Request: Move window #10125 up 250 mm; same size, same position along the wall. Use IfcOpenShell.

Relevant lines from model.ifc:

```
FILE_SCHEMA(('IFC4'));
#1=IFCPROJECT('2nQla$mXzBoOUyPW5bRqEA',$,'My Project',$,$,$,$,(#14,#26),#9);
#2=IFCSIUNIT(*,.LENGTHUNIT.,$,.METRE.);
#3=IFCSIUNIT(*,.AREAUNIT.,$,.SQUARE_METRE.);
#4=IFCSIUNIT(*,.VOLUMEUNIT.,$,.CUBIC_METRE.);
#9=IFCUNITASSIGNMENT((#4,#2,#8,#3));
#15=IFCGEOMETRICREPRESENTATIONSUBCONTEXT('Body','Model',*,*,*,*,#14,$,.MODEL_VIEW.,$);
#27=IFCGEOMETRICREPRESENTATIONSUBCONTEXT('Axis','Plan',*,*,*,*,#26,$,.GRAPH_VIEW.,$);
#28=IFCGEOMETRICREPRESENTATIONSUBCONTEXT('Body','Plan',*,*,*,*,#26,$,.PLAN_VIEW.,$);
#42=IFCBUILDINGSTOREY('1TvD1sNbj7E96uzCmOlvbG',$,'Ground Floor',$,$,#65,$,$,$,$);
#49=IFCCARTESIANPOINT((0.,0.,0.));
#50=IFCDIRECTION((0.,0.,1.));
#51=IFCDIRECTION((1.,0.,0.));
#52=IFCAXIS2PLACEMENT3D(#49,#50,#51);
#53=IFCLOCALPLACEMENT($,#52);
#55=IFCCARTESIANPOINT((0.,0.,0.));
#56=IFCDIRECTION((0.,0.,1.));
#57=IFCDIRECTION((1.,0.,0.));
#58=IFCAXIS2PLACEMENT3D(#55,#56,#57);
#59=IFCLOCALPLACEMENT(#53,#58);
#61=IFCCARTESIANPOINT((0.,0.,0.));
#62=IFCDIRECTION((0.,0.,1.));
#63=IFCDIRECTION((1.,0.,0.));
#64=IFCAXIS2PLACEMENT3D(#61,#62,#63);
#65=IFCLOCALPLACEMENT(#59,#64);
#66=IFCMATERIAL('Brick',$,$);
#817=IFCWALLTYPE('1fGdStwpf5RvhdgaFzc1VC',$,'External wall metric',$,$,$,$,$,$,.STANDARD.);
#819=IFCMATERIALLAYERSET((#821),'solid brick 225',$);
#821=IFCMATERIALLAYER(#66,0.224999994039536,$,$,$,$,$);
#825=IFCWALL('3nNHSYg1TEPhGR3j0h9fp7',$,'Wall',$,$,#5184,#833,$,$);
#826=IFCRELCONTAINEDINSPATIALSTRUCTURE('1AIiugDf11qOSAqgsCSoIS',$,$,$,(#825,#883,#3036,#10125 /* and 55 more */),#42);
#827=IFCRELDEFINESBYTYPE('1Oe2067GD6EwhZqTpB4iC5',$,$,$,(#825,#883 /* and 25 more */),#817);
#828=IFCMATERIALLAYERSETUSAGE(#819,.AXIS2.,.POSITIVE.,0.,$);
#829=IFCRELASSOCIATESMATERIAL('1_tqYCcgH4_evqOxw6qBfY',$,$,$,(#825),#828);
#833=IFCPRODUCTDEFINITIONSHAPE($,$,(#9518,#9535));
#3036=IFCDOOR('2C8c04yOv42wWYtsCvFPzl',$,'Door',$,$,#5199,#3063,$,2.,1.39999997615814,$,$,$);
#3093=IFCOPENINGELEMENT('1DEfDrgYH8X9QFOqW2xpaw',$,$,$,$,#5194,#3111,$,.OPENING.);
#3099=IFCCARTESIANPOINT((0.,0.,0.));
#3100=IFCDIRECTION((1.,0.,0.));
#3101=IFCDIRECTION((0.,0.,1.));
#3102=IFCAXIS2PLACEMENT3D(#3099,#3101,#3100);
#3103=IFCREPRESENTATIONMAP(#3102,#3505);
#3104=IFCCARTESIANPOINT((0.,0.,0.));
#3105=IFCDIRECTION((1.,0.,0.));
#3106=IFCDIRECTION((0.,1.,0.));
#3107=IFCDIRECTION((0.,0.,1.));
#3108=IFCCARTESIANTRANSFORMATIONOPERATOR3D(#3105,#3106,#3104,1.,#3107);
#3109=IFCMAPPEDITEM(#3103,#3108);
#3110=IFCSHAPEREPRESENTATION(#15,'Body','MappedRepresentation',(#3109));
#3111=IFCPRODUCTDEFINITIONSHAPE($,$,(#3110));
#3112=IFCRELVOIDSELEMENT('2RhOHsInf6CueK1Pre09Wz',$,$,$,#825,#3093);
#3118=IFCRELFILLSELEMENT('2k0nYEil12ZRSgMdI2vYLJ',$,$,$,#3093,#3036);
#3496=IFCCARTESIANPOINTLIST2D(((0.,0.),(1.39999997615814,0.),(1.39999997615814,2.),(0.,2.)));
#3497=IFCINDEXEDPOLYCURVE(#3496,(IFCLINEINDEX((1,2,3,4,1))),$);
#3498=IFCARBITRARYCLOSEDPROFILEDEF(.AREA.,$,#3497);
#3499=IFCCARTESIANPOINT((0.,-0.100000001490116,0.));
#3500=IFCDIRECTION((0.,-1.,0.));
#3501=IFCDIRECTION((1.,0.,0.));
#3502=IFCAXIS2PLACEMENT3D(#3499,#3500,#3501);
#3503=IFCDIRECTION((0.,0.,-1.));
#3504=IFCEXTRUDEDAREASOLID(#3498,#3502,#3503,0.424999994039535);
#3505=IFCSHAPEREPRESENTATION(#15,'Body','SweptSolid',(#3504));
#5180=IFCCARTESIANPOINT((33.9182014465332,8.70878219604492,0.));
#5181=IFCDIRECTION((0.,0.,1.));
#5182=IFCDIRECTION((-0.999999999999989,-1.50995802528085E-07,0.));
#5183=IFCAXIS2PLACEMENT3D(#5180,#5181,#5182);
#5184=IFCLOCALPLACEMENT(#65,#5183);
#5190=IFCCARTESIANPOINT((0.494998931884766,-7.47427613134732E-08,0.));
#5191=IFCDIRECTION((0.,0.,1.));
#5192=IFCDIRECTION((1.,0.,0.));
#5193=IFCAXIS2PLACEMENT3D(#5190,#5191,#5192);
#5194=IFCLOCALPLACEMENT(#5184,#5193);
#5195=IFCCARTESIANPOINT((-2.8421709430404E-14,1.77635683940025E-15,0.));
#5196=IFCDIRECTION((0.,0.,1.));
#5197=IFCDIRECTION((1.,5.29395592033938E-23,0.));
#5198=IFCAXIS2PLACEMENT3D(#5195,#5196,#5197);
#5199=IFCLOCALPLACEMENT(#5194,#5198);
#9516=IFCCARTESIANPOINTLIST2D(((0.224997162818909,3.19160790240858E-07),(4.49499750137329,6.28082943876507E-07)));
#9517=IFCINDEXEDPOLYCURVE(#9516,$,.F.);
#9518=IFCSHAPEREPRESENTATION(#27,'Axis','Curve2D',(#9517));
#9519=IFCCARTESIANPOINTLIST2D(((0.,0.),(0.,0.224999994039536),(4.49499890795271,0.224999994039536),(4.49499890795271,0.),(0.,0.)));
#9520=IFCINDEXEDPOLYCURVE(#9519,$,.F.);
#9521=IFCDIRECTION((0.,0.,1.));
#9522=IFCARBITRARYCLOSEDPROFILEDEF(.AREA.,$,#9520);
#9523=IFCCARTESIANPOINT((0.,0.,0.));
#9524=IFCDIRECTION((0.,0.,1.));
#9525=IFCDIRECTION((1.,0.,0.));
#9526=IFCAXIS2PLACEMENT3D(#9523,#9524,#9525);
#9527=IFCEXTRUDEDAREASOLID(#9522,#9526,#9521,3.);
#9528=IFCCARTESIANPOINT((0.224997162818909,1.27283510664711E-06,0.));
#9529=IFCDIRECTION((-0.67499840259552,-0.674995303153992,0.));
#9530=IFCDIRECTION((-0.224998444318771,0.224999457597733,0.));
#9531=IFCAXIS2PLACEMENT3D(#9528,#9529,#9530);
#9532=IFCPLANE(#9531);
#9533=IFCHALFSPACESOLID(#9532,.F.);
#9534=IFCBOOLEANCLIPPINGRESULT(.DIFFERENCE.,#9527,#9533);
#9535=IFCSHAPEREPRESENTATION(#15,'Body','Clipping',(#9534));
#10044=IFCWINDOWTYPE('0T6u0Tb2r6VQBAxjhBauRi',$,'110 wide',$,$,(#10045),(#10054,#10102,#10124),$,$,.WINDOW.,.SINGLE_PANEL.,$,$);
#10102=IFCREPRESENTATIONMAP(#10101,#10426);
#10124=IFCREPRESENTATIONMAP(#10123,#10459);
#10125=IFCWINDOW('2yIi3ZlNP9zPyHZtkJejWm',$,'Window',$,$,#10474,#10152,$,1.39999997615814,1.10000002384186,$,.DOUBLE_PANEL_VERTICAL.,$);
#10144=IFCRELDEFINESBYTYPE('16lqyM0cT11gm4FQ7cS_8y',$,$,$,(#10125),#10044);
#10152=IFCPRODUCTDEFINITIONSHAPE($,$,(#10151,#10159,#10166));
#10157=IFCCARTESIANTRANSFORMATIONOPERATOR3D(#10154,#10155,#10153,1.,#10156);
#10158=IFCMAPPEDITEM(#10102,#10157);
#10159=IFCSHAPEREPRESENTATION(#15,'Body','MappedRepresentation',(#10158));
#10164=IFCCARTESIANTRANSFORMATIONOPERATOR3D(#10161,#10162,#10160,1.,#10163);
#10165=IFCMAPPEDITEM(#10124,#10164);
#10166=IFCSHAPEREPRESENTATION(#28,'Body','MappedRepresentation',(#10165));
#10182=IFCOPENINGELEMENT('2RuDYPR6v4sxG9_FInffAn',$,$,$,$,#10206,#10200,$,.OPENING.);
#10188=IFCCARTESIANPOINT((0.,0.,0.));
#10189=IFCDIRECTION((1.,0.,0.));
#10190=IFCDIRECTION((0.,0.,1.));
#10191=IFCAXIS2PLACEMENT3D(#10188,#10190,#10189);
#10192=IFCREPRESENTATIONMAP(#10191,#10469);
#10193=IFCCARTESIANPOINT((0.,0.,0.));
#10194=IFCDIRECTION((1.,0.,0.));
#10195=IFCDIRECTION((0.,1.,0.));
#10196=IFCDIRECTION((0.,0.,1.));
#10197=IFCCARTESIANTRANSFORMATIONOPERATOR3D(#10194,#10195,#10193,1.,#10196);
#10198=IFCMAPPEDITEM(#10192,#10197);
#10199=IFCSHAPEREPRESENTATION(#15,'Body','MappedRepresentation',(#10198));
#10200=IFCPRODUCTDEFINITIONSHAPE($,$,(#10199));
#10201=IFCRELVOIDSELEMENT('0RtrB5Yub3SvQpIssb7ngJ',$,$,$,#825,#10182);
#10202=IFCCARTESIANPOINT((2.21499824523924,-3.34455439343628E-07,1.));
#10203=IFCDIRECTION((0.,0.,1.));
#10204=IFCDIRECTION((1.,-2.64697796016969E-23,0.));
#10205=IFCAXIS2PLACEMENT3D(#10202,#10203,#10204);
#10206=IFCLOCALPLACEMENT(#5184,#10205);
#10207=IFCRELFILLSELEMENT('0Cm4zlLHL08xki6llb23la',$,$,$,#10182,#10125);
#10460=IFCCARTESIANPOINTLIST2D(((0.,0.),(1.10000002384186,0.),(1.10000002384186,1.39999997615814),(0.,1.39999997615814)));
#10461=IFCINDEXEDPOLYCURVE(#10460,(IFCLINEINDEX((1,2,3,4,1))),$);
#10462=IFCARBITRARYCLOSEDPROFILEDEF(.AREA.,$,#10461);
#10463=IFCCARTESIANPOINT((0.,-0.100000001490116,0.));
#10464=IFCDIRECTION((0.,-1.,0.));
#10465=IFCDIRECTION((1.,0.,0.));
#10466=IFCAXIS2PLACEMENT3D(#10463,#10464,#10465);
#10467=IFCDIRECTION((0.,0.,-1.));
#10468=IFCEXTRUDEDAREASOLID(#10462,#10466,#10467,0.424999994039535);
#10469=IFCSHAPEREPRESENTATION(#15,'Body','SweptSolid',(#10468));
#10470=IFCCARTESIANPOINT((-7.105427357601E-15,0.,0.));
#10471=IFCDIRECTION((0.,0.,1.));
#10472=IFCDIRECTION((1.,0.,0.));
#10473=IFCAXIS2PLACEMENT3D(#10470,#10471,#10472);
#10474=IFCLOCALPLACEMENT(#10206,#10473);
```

```python
import numpy as np
import ifcopenshell
import ifcopenshell.api.geometry
import ifcopenshell.util.placement
import ifcopenshell.util.unit

model = ifcopenshell.open("model.ifc")
unit_scale = ifcopenshell.util.unit.calculate_unit_scale(model)

window = model.by_guid("2yIi3ZlNP9zPyHZtkJejWm")
opening = window.FillsVoids[0].RelatingOpeningElement
dz = 0.25

shift = np.array([0.0, 0.0, dz])
# The window is placed relative to its opening, so it follows when the opening moves.
matrix = ifcopenshell.util.placement.get_local_placement(opening.ObjectPlacement)
matrix[:3, 3] += shift
ifcopenshell.api.geometry.edit_object_placement(
    model, product=opening, matrix=matrix, is_si=False, should_transform_children=True
)

print(f"moved by {dz * unit_scale:+.3f} m")

model.write("model-out.ifc")
```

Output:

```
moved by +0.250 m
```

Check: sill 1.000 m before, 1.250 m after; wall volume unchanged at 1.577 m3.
